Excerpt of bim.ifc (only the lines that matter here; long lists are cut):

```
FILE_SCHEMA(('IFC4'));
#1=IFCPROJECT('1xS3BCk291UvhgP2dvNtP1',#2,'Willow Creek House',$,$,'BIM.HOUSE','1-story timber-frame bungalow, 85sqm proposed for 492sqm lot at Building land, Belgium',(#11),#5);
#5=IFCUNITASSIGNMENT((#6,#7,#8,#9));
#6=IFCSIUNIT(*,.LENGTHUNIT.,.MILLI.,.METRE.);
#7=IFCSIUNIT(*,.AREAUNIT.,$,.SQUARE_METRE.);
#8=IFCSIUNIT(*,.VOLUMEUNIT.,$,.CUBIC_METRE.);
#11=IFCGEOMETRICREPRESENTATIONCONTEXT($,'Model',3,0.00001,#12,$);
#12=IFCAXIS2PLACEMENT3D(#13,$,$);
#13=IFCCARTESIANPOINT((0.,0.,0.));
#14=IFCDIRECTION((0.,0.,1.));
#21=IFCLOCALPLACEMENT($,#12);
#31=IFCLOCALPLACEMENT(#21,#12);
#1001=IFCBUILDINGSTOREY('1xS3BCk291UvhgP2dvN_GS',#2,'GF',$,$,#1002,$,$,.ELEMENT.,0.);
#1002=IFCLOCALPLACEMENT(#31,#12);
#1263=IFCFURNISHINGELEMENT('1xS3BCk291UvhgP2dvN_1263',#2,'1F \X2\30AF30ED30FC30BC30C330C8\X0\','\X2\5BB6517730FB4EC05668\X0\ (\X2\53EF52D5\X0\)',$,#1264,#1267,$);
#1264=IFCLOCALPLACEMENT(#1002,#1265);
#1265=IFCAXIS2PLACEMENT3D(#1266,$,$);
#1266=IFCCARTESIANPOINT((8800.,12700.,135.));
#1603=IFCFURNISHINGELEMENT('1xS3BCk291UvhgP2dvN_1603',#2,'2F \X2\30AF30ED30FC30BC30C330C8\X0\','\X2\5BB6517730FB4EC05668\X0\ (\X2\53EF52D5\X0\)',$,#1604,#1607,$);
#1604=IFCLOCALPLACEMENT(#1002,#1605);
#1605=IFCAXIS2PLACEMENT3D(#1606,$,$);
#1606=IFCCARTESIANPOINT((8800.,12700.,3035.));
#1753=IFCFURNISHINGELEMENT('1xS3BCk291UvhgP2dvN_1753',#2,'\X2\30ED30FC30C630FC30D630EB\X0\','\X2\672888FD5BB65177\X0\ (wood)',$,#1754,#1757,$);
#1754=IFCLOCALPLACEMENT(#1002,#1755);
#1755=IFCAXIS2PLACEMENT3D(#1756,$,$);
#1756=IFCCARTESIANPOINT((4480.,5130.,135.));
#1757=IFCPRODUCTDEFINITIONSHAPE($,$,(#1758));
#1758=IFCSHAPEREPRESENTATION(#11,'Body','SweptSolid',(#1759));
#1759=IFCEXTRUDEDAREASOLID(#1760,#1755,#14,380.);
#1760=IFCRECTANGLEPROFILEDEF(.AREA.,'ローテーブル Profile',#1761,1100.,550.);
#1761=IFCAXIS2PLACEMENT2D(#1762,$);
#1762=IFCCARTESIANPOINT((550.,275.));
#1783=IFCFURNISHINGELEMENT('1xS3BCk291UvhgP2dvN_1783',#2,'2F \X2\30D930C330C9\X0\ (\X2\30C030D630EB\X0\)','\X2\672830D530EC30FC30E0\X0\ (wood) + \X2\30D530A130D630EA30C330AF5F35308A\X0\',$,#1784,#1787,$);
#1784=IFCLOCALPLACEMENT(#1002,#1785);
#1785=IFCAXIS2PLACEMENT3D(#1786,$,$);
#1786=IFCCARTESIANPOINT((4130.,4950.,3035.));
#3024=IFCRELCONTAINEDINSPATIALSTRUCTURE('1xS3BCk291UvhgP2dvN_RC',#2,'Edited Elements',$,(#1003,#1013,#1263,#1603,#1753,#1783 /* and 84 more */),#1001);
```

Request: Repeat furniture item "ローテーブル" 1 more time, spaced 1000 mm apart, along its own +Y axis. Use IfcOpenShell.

```python
import ifcopenshell
import ifcopenshell.api.geometry
import ifcopenshell.api.root
import ifcopenshell.util.element
import ifcopenshell.util.placement

model = ifcopenshell.open("bim.ifc")


def reuse_history(source, copy):
    """copy_class also copies each property set's owner history, people and application; keep the originals."""
    for rel in copy.IsDefinedBy:
        if rel.is_a("IfcRelDefinesByProperties") and (history := rel.RelatingPropertyDefinition.OwnerHistory):
            rel.RelatingPropertyDefinition.OwnerHistory = source.OwnerHistory
            ifcopenshell.util.element.remove_deep2(model, history)


source = model.by_guid("1xS3BCk291UvhgP2dvN_1753")
base = ifcopenshell.util.placement.get_local_placement(source.ObjectPlacement)
step = base[:3, 1] * 1000.0

for i in range(1, 2):
    copy = ifcopenshell.api.root.copy_class(model, product=source)
    copy.Representation = ifcopenshell.util.element.copy_deep(
        model, source.Representation, exclude=["IfcGeometricRepresentationContext", "IfcRepresentationMap"]
    )
    reuse_history(source, copy)
    matrix = base.copy()
    matrix[:3, 3] += i * step
    print("added at", matrix[:3, 3].round(3) + 0.0)
    ifcopenshell.api.geometry.edit_object_placement(model, product=copy, matrix=matrix, is_si=False)

model.write("bim_edited.ifc")
```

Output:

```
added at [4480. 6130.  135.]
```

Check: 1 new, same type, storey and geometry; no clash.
